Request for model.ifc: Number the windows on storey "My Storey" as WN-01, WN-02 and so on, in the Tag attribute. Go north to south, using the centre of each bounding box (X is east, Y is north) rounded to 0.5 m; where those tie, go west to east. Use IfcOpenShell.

First a look at what the model holds.

```python
import ifcopenshell
import ifcopenshell.util.element
import ifcopenshell.util.placement

model = ifcopenshell.open("model.ifc")
print(model.schema)
storey = next(s for s in model.by_type("IfcBuildingStorey") if s.Name == "My Storey")
windows = [e for e in ifcopenshell.util.element.get_decomposition(storey) if e.is_a("IfcWindow")]
for e in sorted(windows, key=lambda e: e.id()):
    origin = ifcopenshell.util.placement.get_local_placement(e.ObjectPlacement)[:3, 3]
    print(e.id(), e.Tag, e.Name, origin.round(2) + 0.0, sep=" | ")
```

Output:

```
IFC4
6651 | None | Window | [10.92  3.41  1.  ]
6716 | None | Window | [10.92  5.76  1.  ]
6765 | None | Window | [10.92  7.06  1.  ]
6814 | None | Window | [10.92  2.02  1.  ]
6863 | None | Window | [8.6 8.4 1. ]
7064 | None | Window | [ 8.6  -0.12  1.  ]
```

```python
import ifcopenshell
import ifcopenshell.geom
import ifcopenshell.util.element
import ifcopenshell.util.shape

model = ifcopenshell.open("model.ifc")
settings = ifcopenshell.geom.settings()
settings.set("use-world-coords", True)


def centre(element):
    shape = ifcopenshell.geom.create_shape(settings, element)
    return ifcopenshell.util.shape.get_bbox_centroid(shape.geometry)


storey = next(s for s in model.by_type("IfcBuildingStorey") if s.Name == "My Storey")
windows = [e for e in ifcopenshell.util.element.get_decomposition(storey) if e.is_a("IfcWindow")]

# Insertion points can sit at a corner or the storey origin, so sort by the geometry (in metres).
centres = {e: centre(e) for e in windows}
windows.sort(key=lambda e: (-round(centres[e][1] / 0.5), centres[e][0]))

for i, e in enumerate(windows, start=1):
    number = f"WN-{i:02d}"
    e.Tag = number
    print(e.id(), number)

model.write("model_updated.ifc")
```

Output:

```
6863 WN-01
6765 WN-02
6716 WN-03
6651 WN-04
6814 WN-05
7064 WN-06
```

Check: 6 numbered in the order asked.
